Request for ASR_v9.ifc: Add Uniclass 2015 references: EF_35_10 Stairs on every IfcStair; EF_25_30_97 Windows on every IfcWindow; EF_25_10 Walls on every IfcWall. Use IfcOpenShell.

First a look at what the model holds.

```python
import ifcopenshell

model = ifcopenshell.open("ASR_v9.ifc")
print(model.schema)
print("classifications:", [c.Name for c in model.by_type("IfcClassification")])
for ifc_class in ("IfcDoor", "IfcRoof", "IfcStair", "IfcWall", "IfcWindow"):
    print(ifc_class, len(model.by_type(ifc_class)))
```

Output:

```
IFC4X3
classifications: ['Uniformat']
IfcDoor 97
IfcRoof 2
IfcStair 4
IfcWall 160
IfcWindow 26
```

```python
import ifcopenshell
import ifcopenshell.api.classification

model = ifcopenshell.open("ASR_v9.ifc")

system = ifcopenshell.api.classification.add_classification(model, classification="Uniclass 2015")

codes = {
    "IfcStair": ("EF_35_10", "Stairs"),
    "IfcWindow": ("EF_25_30_97", "Windows"),
    "IfcWall": ("EF_25_10", "Walls"),
}
for ifc_class, (code, name) in codes.items():
    products = model.by_type(ifc_class)
    ifcopenshell.api.classification.add_reference(
        model, products=products, classification=system, identification=code, name=name
    )
    print(code, len(products))

model.write("ASR_v9_updated.ifc")
```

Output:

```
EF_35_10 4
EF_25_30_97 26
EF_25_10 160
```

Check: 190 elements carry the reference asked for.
